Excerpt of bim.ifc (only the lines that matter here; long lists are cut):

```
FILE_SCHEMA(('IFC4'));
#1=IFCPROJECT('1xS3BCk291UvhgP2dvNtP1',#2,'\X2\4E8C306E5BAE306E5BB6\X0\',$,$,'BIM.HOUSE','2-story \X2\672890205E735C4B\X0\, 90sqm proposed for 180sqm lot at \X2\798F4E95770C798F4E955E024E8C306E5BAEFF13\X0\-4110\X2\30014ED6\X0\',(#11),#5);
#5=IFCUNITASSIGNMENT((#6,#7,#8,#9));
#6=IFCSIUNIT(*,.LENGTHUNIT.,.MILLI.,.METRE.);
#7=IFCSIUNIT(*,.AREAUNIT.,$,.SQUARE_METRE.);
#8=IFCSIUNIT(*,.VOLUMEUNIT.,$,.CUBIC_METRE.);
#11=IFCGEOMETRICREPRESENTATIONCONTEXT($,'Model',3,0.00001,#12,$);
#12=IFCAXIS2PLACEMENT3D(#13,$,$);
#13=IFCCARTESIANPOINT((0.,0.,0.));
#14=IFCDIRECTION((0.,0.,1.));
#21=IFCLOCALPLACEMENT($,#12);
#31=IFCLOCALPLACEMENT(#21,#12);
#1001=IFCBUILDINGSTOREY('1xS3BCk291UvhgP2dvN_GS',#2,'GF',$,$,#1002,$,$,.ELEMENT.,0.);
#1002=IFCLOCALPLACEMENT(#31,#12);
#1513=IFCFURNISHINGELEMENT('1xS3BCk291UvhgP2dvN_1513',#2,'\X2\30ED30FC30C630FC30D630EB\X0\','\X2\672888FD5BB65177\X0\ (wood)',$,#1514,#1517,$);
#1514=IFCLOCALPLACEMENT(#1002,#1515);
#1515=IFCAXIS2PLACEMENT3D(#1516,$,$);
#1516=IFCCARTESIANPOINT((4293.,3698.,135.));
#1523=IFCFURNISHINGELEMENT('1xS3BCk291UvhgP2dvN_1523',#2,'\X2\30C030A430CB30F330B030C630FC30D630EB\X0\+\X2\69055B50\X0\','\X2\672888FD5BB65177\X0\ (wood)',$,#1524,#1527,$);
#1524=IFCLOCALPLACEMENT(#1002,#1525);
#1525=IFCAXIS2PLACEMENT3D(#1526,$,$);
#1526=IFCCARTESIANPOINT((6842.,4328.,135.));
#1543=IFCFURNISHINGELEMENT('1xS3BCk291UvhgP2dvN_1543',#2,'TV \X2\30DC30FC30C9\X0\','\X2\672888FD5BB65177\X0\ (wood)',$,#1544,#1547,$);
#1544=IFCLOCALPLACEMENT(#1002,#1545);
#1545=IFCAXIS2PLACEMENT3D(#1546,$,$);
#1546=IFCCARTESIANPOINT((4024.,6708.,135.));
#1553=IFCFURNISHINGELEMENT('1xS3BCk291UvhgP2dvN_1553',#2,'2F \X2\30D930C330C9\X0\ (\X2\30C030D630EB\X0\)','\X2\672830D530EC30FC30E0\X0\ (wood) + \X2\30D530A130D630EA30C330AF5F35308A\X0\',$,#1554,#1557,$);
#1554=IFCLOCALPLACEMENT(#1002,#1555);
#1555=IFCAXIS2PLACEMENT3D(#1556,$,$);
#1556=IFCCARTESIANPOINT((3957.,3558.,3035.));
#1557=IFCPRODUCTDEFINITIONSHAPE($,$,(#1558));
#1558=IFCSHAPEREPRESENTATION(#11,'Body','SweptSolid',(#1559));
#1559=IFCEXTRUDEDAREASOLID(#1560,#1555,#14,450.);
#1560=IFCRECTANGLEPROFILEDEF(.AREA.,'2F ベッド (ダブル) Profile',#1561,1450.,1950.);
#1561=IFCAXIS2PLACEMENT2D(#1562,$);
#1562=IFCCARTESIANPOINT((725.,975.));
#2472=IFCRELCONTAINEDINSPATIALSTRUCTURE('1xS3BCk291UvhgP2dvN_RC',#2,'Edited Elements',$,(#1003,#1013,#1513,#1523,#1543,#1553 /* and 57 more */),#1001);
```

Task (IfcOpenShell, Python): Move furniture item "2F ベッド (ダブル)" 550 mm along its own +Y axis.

```python
import ifcopenshell
import ifcopenshell.api.geometry
import ifcopenshell.util.placement
import ifcopenshell.util.unit

model = ifcopenshell.open("bim.ifc")
unit_scale = ifcopenshell.util.unit.calculate_unit_scale(model)

item = model.by_guid("1xS3BCk291UvhgP2dvN_1553")
matrix = ifcopenshell.util.placement.get_local_placement(item.ObjectPlacement)
matrix[:3, 3] += matrix[:3, 1] * 0.55 / unit_scale
ifcopenshell.api.geometry.edit_object_placement(model, product=item, matrix=matrix, is_si=False)

print(ifcopenshell.util.placement.get_local_placement(item.ObjectPlacement).round(3) + 0.0)

model.write("bim_rev.ifc")
```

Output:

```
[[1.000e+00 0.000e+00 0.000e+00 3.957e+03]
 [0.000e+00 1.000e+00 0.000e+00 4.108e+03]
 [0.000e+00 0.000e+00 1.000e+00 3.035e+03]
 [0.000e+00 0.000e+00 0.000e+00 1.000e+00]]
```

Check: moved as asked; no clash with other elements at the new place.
